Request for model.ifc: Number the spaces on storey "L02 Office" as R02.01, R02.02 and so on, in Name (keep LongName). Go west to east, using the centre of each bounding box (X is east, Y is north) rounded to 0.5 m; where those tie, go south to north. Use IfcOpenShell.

First a look at what the model holds.

```python
import ifcopenshell
import ifcopenshell.util.element
import ifcopenshell.util.placement

model = ifcopenshell.open("model.ifc")
print(model.schema)
storey = next(s for s in model.by_type("IfcBuildingStorey") if s.Name == "L02 Office")
spaces = [e for e in ifcopenshell.util.element.get_decomposition(storey) if e.is_a("IfcSpace")]
for e in sorted(spaces, key=lambda e: e.id()):
    origin = ifcopenshell.util.placement.get_local_placement(e.ObjectPlacement)[:3, 3]
    print(e.id(), e.Name, e.LongName, origin.round(2) + 0.0, sep=" | ")
```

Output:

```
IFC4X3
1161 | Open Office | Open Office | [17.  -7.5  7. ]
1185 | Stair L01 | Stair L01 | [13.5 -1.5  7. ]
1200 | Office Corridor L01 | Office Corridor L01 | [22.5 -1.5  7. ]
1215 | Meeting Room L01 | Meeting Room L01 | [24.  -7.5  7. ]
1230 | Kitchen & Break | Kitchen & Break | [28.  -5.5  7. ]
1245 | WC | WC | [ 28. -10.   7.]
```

```python
import ifcopenshell
import ifcopenshell.geom
import ifcopenshell.util.element
import ifcopenshell.util.shape

model = ifcopenshell.open("model.ifc")
settings = ifcopenshell.geom.settings()
settings.set("use-world-coords", True)


def centre(element):
    shape = ifcopenshell.geom.create_shape(settings, element)
    return ifcopenshell.util.shape.get_bbox_centroid(shape.geometry)


storey = next(s for s in model.by_type("IfcBuildingStorey") if s.Name == "L02 Office")
spaces = [e for e in ifcopenshell.util.element.get_decomposition(storey) if e.is_a("IfcSpace")]

# Insertion points can sit at a corner or the storey origin, so sort by the geometry (in metres).
centres = {e: centre(e) for e in spaces}
spaces.sort(key=lambda e: (round(centres[e][0] / 0.5), centres[e][1]))

for i, e in enumerate(spaces, start=1):
    number = f"R02.{i:02d}"
    e.Name = number
    print(e.id(), number)

model.write("model_v2.ifc")
```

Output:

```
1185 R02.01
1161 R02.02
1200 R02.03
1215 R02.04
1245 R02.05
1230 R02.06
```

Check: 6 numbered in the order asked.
